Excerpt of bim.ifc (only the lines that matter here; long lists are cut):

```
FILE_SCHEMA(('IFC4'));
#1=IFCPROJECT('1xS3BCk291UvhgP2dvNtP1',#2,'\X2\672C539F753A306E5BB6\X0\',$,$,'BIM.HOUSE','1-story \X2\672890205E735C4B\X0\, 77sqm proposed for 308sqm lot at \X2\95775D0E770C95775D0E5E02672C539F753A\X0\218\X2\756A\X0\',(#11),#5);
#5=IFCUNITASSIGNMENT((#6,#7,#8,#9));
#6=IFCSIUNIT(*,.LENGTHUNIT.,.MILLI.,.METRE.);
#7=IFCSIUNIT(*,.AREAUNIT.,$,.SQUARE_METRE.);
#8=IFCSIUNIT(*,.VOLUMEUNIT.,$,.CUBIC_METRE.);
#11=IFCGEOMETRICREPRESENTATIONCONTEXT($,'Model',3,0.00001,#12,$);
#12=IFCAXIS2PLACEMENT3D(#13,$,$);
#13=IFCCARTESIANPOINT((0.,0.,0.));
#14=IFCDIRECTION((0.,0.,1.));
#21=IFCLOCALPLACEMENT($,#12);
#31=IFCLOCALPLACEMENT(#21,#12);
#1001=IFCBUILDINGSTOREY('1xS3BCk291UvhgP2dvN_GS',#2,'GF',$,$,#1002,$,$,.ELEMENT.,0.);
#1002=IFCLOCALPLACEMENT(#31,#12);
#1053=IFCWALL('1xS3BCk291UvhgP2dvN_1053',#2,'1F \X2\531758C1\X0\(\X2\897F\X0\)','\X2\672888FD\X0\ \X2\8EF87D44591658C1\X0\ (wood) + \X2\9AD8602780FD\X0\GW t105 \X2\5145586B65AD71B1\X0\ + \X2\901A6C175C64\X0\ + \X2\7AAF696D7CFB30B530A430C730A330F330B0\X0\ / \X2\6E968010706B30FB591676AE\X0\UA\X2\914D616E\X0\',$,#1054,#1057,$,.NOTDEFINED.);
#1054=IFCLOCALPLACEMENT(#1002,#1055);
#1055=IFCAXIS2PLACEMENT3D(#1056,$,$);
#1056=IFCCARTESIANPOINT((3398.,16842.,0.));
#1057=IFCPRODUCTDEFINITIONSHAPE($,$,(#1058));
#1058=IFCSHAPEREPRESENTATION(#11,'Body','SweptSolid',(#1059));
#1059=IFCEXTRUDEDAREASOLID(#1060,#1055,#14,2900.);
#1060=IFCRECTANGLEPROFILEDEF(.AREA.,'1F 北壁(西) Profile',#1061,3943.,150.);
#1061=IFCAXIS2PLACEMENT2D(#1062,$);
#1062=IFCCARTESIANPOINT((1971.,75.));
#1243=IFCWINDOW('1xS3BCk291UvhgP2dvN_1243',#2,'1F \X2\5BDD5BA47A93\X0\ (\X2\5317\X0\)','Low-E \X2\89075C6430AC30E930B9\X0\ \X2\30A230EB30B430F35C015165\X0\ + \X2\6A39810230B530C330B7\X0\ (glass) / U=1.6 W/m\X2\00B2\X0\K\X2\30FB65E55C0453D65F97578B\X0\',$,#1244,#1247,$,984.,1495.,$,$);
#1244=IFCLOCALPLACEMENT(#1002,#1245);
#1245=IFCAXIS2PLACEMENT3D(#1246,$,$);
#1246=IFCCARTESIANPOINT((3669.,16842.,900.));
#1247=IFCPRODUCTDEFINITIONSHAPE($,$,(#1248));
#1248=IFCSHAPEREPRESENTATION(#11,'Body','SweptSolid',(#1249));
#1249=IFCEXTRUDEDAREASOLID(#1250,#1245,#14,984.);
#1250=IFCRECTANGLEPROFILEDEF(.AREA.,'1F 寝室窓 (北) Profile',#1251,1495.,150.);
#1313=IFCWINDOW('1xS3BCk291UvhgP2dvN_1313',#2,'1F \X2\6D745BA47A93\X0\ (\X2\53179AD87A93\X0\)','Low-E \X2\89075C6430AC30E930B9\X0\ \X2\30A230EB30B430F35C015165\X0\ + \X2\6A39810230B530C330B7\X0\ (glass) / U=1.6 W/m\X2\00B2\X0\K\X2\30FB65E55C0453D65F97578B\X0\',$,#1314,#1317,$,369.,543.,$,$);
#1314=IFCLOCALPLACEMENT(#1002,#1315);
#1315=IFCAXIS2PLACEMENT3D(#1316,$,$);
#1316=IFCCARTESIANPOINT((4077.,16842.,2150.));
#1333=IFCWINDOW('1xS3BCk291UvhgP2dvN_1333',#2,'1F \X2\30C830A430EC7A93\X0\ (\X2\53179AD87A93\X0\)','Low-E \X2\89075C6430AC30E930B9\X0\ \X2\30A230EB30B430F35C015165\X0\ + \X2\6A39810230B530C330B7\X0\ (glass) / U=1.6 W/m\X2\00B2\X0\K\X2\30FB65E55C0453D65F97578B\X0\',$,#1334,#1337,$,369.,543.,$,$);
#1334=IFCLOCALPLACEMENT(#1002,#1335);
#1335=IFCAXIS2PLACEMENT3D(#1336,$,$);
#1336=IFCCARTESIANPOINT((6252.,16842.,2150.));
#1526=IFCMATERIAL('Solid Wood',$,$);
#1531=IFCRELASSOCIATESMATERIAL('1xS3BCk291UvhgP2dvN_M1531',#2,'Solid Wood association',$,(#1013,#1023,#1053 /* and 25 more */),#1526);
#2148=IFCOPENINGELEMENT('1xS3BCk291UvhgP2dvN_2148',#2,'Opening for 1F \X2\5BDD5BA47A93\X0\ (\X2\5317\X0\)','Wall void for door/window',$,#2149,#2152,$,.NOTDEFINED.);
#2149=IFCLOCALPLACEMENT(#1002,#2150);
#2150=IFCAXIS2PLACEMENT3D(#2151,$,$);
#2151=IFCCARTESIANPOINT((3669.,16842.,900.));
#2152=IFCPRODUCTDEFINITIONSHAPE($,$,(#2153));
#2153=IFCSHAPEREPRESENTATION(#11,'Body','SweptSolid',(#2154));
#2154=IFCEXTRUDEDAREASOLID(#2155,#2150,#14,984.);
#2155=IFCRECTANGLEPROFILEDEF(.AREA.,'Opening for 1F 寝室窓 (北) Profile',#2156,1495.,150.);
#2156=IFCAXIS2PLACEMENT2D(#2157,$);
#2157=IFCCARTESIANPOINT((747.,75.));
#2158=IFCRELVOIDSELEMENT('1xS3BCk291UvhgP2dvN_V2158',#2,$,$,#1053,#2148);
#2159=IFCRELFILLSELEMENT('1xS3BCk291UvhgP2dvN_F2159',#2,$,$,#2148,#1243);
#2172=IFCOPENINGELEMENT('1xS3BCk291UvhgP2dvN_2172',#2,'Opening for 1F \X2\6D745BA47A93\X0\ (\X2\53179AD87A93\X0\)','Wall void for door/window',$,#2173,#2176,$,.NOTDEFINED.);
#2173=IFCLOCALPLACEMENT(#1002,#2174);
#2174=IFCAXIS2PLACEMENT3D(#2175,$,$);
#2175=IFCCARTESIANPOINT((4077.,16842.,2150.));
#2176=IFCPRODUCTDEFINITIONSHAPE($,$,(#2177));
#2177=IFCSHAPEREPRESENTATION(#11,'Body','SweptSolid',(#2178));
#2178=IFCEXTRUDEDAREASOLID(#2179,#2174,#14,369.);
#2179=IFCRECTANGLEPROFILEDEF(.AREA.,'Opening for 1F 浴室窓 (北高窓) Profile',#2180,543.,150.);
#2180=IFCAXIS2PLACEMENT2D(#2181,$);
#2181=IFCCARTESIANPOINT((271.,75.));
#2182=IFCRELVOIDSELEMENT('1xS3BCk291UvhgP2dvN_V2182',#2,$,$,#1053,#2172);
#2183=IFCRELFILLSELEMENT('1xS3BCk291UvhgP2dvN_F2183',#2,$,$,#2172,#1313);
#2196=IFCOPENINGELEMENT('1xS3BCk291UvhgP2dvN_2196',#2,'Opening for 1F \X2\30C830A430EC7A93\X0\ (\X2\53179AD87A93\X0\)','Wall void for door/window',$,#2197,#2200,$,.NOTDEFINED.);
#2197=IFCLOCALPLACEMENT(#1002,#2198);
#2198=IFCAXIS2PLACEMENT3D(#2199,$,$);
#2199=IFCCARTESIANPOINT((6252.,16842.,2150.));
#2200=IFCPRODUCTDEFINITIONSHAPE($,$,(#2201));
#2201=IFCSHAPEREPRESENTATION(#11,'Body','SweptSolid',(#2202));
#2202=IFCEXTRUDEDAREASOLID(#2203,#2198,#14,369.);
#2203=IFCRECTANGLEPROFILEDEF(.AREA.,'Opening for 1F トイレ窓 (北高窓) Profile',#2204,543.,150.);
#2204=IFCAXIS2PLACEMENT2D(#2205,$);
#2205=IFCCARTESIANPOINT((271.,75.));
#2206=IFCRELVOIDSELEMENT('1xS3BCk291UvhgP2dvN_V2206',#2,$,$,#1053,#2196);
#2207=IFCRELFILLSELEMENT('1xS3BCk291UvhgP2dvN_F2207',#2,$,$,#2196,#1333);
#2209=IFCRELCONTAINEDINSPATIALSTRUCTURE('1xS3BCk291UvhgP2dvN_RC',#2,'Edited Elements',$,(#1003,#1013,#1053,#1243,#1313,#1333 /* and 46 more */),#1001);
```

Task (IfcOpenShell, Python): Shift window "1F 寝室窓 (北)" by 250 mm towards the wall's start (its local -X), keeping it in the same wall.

```python
import ifcopenshell
import ifcopenshell.api.geometry
import ifcopenshell.util.placement

model = ifcopenshell.open("bim.ifc")

window = model.by_guid("1xS3BCk291UvhgP2dvN_1243")
opening = window.FillsVoids[0].RelatingOpeningElement
wall = opening.VoidsElements[0].RelatingBuildingElement

wall_matrix = ifcopenshell.util.placement.get_local_placement(wall.ObjectPlacement)
shift = wall_matrix[:3, 0] * -250.0
before = ifcopenshell.util.placement.get_local_placement(window.ObjectPlacement)[:3, 3].copy()

# The window is not placed relative to its opening, so move both.
for product in (opening, window):
    matrix = ifcopenshell.util.placement.get_local_placement(product.ObjectPlacement)
    matrix[:3, 3] += shift
    ifcopenshell.api.geometry.edit_object_placement(model, product=product, matrix=matrix, is_si=False)

after = ifcopenshell.util.placement.get_local_placement(window.ObjectPlacement)[:3, 3]
print("window moved by", (after - before).round(3) + 0.0)

model.write("bim-out.ifc")
```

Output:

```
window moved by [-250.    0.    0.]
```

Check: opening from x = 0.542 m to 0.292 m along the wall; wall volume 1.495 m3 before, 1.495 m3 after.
